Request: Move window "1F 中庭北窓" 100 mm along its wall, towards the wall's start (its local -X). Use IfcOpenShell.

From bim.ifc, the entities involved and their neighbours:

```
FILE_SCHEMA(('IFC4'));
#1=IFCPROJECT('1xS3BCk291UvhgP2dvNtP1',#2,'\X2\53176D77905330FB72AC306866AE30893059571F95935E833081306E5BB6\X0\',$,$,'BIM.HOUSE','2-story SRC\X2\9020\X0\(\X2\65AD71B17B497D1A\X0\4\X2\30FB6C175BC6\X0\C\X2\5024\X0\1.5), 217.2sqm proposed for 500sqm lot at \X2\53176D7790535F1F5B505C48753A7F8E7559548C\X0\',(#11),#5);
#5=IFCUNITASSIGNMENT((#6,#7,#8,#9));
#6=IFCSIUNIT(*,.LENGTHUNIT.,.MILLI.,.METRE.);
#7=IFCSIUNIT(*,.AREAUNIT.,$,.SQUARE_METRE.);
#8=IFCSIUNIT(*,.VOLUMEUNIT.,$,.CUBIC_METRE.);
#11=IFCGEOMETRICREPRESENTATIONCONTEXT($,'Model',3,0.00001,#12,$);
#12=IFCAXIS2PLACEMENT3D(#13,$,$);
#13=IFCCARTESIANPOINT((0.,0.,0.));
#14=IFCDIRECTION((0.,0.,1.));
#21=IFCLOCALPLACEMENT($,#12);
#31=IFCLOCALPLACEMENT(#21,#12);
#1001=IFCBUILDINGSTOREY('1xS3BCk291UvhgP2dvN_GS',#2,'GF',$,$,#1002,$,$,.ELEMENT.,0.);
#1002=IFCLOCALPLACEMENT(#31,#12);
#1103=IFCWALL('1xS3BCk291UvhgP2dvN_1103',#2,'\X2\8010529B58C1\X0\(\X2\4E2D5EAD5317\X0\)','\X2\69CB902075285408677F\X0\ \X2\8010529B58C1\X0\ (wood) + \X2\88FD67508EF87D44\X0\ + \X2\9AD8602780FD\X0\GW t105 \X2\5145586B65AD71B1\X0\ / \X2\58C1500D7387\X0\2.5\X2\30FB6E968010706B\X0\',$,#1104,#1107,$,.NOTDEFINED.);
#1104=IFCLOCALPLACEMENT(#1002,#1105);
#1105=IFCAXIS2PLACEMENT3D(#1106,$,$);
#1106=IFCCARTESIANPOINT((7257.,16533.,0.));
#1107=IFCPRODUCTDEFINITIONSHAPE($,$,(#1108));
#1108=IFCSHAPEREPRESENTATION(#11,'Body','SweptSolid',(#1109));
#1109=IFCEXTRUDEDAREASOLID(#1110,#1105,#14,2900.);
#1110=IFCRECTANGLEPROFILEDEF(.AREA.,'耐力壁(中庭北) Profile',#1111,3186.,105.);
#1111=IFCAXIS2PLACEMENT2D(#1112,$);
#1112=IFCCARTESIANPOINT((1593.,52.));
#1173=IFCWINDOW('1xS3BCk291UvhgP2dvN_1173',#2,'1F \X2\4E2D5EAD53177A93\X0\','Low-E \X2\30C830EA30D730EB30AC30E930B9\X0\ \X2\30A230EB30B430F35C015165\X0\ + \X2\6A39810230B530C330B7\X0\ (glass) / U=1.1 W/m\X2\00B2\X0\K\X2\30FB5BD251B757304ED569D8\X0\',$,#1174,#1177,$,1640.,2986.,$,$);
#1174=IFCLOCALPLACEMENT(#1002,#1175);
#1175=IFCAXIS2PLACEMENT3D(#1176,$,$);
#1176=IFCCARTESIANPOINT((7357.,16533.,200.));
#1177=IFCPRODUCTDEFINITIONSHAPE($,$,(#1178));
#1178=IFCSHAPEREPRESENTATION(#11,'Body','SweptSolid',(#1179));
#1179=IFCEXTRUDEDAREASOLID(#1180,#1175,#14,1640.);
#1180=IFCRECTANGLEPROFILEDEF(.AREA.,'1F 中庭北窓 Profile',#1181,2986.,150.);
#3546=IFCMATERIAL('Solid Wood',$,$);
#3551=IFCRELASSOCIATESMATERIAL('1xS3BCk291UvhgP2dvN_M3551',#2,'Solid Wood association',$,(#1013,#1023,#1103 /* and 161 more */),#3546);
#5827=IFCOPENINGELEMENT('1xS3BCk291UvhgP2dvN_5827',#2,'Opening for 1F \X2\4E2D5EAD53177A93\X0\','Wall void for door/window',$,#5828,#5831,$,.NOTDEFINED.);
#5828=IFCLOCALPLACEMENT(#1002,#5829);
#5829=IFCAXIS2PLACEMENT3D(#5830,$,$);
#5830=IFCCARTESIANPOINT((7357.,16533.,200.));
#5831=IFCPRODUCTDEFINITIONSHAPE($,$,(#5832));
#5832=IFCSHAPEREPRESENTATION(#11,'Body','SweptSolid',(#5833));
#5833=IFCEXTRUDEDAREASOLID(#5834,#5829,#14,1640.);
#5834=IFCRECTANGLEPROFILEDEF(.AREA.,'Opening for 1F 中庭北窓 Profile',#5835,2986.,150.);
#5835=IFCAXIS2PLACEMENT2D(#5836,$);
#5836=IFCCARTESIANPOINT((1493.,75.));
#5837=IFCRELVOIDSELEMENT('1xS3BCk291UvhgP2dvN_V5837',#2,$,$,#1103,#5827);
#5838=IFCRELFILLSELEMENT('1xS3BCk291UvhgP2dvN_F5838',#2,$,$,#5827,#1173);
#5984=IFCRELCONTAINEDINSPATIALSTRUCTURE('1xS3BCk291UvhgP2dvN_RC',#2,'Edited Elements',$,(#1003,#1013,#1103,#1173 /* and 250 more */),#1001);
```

```python
import ifcopenshell
import ifcopenshell.api.geometry
import ifcopenshell.util.placement
import ifcopenshell.util.unit

model = ifcopenshell.open("bim.ifc")
unit_scale = ifcopenshell.util.unit.calculate_unit_scale(model)

window = model.by_guid("1xS3BCk291UvhgP2dvN_1173")
opening = window.FillsVoids[0].RelatingOpeningElement
wall = opening.VoidsElements[0].RelatingBuildingElement

wall_matrix = ifcopenshell.util.placement.get_local_placement(wall.ObjectPlacement)
shift = wall_matrix[:3, 0] * -0.1 / unit_scale
before = ifcopenshell.util.placement.get_local_placement(window.ObjectPlacement)[:3, 3].copy()

# The window is not placed relative to its opening, so move both.
for product in (opening, window):
    matrix = ifcopenshell.util.placement.get_local_placement(product.ObjectPlacement)
    matrix[:3, 3] += shift
    ifcopenshell.api.geometry.edit_object_placement(model, product=product, matrix=matrix, is_si=False)

after = ifcopenshell.util.placement.get_local_placement(window.ObjectPlacement)[:3, 3]
print("window moved by", (after - before).round(3) + 0.0)

model.write("bim_edited.ifc")
```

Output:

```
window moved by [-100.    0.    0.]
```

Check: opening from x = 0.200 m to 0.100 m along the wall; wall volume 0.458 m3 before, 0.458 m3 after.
